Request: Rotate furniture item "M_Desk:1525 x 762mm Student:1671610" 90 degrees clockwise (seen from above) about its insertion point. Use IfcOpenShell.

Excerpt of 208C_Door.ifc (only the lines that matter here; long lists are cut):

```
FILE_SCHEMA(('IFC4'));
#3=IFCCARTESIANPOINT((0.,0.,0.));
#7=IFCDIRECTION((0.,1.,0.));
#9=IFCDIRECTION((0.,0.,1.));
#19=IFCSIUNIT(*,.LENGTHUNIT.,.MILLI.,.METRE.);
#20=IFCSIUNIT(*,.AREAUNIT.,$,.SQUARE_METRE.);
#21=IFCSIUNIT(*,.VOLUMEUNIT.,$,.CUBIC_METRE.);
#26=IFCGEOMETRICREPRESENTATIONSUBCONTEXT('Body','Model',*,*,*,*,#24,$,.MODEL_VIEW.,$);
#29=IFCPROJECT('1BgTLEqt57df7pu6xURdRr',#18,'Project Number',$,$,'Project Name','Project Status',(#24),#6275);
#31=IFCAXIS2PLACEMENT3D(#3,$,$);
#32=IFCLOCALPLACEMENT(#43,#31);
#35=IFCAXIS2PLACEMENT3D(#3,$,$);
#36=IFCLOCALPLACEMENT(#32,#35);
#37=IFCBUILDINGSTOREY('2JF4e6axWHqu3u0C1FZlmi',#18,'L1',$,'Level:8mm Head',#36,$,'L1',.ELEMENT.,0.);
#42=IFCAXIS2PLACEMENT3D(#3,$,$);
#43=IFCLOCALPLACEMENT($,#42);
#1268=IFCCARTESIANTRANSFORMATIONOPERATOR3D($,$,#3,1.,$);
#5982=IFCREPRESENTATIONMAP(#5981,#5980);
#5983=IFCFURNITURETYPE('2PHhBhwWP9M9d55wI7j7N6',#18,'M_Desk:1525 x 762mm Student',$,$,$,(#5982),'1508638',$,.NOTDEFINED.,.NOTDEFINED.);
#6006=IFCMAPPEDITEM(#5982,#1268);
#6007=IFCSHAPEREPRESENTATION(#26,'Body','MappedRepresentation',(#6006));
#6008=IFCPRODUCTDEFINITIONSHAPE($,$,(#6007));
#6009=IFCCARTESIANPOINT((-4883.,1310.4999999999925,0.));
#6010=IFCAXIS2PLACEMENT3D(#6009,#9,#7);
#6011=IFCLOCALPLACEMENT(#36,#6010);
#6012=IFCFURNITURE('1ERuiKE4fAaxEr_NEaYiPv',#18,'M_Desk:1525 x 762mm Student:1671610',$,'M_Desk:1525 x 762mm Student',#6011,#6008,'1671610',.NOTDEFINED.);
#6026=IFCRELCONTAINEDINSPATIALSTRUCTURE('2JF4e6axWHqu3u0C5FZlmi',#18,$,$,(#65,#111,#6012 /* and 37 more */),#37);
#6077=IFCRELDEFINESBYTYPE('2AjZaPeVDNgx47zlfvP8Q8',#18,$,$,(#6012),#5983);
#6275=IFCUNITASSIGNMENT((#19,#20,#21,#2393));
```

```python
import ifcopenshell
import ifcopenshell.api.geometry
import ifcopenshell.util.placement

model = ifcopenshell.open("208C_Door.ifc")

item = model.by_id(6012)
matrix = ifcopenshell.util.placement.get_local_placement(item.ObjectPlacement)
matrix = matrix @ ifcopenshell.util.placement.rotation(-90, "Z")
ifcopenshell.api.geometry.edit_object_placement(model, product=item, matrix=matrix, is_si=False)

print(ifcopenshell.util.placement.get_local_placement(item.ObjectPlacement).round(3) + 0.0)

model.write("208C_Door-out.ifc")
```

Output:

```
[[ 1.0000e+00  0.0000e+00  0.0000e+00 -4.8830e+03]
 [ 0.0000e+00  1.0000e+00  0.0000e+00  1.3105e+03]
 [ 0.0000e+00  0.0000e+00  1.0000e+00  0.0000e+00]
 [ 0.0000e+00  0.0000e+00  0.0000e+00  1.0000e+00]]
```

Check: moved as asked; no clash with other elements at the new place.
